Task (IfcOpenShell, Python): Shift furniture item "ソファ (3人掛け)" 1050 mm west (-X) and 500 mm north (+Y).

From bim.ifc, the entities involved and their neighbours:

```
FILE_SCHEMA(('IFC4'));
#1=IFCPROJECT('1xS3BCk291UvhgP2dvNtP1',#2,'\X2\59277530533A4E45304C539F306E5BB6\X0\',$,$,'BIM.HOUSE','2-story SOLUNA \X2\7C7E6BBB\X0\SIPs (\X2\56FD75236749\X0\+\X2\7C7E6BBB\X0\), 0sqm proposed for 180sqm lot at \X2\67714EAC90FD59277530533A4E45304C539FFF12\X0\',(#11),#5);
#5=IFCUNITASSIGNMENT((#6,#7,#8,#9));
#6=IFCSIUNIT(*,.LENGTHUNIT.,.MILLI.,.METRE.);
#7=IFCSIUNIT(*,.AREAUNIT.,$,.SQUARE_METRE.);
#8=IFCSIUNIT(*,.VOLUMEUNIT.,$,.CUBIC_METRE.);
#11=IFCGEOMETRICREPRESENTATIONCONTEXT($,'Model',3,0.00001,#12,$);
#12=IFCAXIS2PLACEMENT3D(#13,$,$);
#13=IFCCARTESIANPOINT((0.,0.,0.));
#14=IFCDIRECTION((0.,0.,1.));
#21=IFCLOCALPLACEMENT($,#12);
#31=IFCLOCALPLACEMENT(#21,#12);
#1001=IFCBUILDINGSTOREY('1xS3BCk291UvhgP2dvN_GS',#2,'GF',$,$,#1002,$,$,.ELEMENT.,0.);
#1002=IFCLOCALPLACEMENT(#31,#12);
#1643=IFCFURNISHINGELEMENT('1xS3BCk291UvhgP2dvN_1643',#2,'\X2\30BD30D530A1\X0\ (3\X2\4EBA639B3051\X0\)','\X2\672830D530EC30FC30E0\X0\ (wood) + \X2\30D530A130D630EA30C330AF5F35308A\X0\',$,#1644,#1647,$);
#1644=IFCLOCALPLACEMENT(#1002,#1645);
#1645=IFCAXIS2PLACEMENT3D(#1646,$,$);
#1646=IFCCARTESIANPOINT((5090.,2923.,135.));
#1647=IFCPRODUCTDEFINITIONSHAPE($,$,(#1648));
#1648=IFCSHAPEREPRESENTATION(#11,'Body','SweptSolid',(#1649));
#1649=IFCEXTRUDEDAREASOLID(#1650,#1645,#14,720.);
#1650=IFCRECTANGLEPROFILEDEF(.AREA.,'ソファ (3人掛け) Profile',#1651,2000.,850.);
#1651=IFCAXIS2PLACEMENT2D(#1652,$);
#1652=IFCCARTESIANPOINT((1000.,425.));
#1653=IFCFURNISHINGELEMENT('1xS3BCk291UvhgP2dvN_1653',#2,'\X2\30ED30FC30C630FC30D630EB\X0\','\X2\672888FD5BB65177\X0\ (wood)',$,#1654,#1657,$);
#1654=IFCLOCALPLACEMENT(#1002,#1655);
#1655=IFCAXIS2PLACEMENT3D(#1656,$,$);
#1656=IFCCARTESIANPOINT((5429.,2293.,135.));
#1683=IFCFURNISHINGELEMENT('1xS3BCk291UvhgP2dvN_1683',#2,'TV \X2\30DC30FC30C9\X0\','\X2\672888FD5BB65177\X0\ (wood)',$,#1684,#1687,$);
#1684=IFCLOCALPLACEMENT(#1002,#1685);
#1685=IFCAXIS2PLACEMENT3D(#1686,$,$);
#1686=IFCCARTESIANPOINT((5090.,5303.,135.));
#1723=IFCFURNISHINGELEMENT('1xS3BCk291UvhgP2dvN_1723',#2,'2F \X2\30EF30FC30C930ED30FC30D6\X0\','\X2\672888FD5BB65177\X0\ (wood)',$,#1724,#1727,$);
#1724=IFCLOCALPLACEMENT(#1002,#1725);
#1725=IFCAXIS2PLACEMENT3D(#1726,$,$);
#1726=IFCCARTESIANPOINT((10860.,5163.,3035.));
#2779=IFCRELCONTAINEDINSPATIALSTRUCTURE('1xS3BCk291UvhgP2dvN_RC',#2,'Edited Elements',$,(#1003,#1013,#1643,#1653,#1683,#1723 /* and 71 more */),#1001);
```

```python
import ifcopenshell
import ifcopenshell.api.geometry
import ifcopenshell.util.placement
import ifcopenshell.util.unit

model = ifcopenshell.open("bim.ifc")
unit_scale = ifcopenshell.util.unit.calculate_unit_scale(model)

item = model.by_guid("1xS3BCk291UvhgP2dvN_1643")
matrix = ifcopenshell.util.placement.get_local_placement(item.ObjectPlacement)
matrix[0, 3] -= 1.05 / unit_scale
matrix[1, 3] += 0.5 / unit_scale
ifcopenshell.api.geometry.edit_object_placement(model, product=item, matrix=matrix, is_si=False)

print(ifcopenshell.util.placement.get_local_placement(item.ObjectPlacement).round(3) + 0.0)

model.write("bim_v2.ifc")
```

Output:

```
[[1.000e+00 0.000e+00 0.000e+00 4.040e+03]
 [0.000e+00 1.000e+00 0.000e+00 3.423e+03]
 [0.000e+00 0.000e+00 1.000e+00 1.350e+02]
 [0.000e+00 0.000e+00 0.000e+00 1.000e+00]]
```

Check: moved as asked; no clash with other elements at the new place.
